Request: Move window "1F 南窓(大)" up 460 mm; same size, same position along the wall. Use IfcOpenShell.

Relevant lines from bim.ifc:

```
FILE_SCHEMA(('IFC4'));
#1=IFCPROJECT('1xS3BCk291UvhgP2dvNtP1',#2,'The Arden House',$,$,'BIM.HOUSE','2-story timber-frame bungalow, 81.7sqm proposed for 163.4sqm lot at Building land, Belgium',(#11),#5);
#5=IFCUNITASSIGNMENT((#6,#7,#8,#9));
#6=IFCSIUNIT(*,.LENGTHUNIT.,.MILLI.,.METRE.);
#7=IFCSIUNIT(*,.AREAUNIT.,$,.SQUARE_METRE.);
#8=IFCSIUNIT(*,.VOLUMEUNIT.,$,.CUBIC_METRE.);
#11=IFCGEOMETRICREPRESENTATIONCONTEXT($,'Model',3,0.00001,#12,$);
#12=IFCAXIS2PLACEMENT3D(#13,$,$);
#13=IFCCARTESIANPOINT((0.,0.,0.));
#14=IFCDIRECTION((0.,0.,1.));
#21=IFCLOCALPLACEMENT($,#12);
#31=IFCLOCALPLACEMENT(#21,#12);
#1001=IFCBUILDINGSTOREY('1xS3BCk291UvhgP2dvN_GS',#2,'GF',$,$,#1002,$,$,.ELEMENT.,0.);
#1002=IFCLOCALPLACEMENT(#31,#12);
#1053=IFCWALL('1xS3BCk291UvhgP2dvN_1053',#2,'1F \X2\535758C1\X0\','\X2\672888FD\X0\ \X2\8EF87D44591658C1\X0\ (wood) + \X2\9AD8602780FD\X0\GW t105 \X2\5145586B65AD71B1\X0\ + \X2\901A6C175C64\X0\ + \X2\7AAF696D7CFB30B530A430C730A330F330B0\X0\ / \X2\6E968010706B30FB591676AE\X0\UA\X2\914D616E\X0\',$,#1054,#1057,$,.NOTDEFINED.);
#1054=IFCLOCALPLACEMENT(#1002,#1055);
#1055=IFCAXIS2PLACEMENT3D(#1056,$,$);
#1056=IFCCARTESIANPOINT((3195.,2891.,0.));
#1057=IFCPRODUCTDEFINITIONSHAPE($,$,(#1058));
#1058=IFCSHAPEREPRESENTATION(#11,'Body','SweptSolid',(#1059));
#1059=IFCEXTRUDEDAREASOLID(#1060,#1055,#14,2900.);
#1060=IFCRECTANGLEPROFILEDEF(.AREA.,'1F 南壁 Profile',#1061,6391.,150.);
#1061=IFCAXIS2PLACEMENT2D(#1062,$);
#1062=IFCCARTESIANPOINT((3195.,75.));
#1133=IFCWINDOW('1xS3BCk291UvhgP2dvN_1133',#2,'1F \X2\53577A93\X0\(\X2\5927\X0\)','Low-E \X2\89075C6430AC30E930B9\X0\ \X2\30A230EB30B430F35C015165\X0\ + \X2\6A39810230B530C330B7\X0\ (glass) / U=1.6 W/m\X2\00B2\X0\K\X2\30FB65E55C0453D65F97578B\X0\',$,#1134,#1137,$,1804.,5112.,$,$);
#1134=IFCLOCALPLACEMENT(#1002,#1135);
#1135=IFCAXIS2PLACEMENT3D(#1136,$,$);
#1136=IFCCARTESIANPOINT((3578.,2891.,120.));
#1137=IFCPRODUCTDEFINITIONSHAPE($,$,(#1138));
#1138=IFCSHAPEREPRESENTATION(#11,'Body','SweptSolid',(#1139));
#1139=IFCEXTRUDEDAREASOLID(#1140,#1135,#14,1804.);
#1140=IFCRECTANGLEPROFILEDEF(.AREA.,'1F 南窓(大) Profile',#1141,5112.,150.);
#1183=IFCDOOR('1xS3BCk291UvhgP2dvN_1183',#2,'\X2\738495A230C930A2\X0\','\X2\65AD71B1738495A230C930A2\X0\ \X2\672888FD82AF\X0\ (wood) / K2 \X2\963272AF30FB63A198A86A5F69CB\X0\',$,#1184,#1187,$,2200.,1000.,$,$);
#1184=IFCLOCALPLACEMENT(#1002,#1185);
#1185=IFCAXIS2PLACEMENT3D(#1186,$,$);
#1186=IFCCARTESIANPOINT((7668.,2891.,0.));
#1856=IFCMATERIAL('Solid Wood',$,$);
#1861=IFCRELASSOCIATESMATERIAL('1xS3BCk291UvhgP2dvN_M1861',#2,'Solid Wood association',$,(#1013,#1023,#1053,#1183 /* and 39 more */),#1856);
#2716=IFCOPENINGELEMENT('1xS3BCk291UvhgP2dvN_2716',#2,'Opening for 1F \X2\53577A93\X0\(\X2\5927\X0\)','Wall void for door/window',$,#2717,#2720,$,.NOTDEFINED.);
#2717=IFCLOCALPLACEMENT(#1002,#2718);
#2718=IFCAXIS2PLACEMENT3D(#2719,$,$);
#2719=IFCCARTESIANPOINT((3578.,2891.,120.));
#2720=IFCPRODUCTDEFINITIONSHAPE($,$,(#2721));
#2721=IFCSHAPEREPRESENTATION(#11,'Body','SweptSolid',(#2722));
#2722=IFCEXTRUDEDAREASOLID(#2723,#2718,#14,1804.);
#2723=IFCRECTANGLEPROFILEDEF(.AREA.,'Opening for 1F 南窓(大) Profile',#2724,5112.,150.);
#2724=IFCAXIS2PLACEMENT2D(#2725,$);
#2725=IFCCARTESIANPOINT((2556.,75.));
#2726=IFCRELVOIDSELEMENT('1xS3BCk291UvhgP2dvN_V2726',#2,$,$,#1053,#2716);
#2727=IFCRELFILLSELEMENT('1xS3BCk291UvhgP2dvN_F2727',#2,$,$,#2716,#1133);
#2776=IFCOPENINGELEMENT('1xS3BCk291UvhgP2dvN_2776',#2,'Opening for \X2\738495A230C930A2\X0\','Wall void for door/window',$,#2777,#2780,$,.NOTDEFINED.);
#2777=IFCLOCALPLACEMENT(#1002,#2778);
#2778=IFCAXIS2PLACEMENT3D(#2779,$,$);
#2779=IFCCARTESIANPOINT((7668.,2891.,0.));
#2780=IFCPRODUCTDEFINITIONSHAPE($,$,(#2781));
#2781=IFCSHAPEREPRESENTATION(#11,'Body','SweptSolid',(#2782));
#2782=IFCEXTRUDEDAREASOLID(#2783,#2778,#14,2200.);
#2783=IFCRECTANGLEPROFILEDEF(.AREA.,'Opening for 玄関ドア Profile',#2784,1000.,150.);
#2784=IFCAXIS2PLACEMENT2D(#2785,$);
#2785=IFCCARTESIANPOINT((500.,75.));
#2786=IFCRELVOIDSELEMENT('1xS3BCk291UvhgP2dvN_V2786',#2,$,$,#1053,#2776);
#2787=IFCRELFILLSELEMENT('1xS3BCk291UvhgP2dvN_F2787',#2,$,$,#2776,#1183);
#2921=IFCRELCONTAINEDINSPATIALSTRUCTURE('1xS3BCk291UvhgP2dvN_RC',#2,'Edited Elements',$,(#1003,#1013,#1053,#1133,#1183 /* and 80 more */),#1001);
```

```python
import numpy as np
import ifcopenshell
import ifcopenshell.api.geometry
import ifcopenshell.util.placement
import ifcopenshell.util.unit

model = ifcopenshell.open("bim.ifc")
unit_scale = ifcopenshell.util.unit.calculate_unit_scale(model)

window = model.by_guid("1xS3BCk291UvhgP2dvN_1133")
opening = window.FillsVoids[0].RelatingOpeningElement
dz = 460.0

shift = np.array([0.0, 0.0, dz])
# The window is not placed relative to its opening, so move both.
for product in (opening, window):
    matrix = ifcopenshell.util.placement.get_local_placement(product.ObjectPlacement)
    matrix[:3, 3] += shift
    ifcopenshell.api.geometry.edit_object_placement(model, product=product, matrix=matrix, is_si=False)

print(f"moved by {dz * unit_scale:+.3f} m")

model.write("bim-out.ifc")
```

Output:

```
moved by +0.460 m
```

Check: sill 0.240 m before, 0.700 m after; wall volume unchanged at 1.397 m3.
